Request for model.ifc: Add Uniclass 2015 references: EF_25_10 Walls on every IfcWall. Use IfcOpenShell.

First a look at what the model holds.

```python
import ifcopenshell

model = ifcopenshell.open("model.ifc")
print(model.schema)
print("classifications:", [c.Name for c in model.by_type("IfcClassification")])
for ifc_class in ("IfcDoor", "IfcRoof", "IfcStair", "IfcWall", "IfcWindow"):
    print(ifc_class, len(model.by_type(ifc_class)))
```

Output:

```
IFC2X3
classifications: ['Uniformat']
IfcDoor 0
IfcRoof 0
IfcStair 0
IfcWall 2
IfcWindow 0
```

```python
import ifcopenshell
import ifcopenshell.api.classification

model = ifcopenshell.open("model.ifc")

# IFC2X3 requires Source and Edition and has no link from the project to the system.
system = model.create_entity("IfcClassification", Source="NBS", Edition="2015", Name="Uniclass 2015")

codes = {
    "IfcWall": ("EF_25_10", "Walls"),
}
for ifc_class, (code, name) in codes.items():
    products = model.by_type(ifc_class)
    ifcopenshell.api.classification.add_reference(
        model, products=products, classification=system, identification=code, name=name
    )
    print(code, len(products))

model.write("model_edited.ifc")
```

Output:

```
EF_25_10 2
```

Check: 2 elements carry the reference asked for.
